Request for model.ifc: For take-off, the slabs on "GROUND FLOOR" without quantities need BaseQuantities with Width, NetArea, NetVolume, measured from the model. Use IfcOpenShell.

First a look at what the model holds.

```python
import ifcopenshell
import ifcopenshell.util.element
import ifcopenshell.util.unit

model = ifcopenshell.open("model.ifc")
print(model.schema)
for unit_type in ("LENGTHUNIT", "AREAUNIT", "VOLUMEUNIT"):
    print(unit_type, ifcopenshell.util.unit.calculate_unit_scale(model, unit_type))
storey = next(s for s in model.by_type("IfcBuildingStorey") if s.Name == "GROUND FLOOR")
slabs = [e for e in ifcopenshell.util.element.get_decomposition(storey) if e.is_a("IfcSlab")]
for e in sorted(slabs, key=lambda e: e.id()):
    print(e.id(), e.is_a(), e.Name, list(ifcopenshell.util.element.get_psets(e, qtos_only=True)), sep=" | ")
```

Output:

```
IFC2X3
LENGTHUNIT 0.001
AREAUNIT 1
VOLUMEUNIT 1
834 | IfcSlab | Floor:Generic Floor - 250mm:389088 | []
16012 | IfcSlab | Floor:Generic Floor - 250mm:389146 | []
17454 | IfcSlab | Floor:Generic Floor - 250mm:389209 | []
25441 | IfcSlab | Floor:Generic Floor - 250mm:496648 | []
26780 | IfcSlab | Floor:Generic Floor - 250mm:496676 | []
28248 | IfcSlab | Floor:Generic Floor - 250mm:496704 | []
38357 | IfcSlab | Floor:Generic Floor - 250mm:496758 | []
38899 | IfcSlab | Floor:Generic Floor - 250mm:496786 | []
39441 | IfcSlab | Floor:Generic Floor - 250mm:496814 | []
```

```python
import ifcopenshell
import ifcopenshell.api.pset
import ifcopenshell.geom
import ifcopenshell.util.element
import ifcopenshell.util.shape
import ifcopenshell.util.unit

model = ifcopenshell.open("model.ifc")
unit_scale = ifcopenshell.util.unit.calculate_unit_scale(model)
area_scale = ifcopenshell.util.unit.calculate_unit_scale(model, "AREAUNIT")
volume_scale = ifcopenshell.util.unit.calculate_unit_scale(model, "VOLUMEUNIT")
settings = ifcopenshell.geom.settings()

storey = next(s for s in model.by_type("IfcBuildingStorey") if s.Name == "GROUND FLOOR")
slabs = [e for e in ifcopenshell.util.element.get_decomposition(storey) if e.is_a("IfcSlab")]

for e in sorted(slabs, key=lambda e: e.id()):
    if ifcopenshell.util.element.get_psets(e, qtos_only=True, should_inherit=False):
        continue
    # Geometry comes back in metres, in the element's own axes.
    shape = ifcopenshell.geom.create_shape(settings, e)
    values = {
        "Width": ifcopenshell.util.shape.get_z(shape.geometry) / unit_scale,
        "NetArea": ifcopenshell.util.shape.get_footprint_area(shape.geometry) / area_scale,
        "NetVolume": ifcopenshell.util.shape.get_volume(shape.geometry) / volume_scale,
    }
    qto = ifcopenshell.api.pset.add_qto(model, product=e, name="BaseQuantities")
    ifcopenshell.api.pset.edit_qto(model, qto=qto, properties=values)
    print(e.id(), {k: round(v, 3) for k, v in values.items()})

model.write("model_updated.ifc")
```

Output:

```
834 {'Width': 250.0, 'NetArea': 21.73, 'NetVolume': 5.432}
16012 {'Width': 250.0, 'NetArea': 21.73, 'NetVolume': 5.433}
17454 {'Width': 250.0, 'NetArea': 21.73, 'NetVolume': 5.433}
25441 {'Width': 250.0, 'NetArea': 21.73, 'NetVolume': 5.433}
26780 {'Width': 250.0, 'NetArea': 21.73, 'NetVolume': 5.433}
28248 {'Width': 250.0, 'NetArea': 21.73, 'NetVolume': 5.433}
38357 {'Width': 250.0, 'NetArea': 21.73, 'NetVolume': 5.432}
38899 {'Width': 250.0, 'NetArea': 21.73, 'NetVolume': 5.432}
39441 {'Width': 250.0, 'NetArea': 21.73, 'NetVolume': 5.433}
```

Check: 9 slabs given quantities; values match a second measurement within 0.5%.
